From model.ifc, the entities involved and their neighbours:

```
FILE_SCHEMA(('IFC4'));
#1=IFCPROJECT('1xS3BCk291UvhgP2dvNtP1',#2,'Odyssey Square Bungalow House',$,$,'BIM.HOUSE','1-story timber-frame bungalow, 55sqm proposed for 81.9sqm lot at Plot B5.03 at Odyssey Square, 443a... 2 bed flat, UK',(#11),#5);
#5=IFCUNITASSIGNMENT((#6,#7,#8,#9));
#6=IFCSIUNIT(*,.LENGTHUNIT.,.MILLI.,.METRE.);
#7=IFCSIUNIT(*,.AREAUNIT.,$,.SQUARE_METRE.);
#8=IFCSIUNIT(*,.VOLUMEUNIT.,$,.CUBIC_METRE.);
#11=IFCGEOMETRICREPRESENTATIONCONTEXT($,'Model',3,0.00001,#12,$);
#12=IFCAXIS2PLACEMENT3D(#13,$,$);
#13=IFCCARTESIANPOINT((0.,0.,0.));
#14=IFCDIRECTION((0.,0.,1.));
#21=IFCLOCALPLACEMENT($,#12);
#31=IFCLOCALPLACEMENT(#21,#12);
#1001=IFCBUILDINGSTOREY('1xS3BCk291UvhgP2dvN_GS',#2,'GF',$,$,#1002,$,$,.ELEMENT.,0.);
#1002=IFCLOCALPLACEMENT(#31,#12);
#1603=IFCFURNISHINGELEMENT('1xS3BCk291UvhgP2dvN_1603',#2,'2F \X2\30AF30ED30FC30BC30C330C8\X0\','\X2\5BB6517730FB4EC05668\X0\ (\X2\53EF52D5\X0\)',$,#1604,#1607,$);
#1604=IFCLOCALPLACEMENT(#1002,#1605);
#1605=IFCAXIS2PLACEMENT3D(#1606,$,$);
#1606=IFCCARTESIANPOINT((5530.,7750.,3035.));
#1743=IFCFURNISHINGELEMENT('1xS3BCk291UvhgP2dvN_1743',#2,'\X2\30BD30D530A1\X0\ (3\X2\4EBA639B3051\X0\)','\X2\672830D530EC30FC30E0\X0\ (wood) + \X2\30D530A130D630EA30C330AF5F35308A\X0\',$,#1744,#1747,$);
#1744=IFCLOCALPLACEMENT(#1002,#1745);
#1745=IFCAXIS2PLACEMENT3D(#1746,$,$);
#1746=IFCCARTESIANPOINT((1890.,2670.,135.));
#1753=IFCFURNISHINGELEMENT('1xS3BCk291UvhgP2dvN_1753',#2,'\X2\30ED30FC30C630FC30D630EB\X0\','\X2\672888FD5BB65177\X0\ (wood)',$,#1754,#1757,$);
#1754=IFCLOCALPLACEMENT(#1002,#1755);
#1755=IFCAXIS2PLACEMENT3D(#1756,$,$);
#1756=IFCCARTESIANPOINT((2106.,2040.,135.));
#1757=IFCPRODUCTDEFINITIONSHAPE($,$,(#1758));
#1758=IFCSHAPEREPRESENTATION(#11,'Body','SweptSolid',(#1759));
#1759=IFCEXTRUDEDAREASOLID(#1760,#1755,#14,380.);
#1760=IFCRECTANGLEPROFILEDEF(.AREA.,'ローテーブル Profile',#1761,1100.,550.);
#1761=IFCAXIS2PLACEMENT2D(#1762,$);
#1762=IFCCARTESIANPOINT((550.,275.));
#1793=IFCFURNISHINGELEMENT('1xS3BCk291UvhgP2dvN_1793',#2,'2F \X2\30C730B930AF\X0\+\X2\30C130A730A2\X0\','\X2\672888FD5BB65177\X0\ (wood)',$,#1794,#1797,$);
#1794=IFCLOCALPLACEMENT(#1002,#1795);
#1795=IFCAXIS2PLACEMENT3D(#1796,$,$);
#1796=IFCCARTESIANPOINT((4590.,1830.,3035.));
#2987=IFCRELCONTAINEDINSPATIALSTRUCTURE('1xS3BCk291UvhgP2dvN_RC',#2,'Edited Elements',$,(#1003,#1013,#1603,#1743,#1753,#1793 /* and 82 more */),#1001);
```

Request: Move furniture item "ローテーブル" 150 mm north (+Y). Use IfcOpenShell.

```python
import ifcopenshell
import ifcopenshell.api.geometry
import ifcopenshell.util.placement

model = ifcopenshell.open("model.ifc")

item = model.by_guid("1xS3BCk291UvhgP2dvN_1753")
matrix = ifcopenshell.util.placement.get_local_placement(item.ObjectPlacement)
matrix[1, 3] += 150.0
ifcopenshell.api.geometry.edit_object_placement(model, product=item, matrix=matrix, is_si=False)

print(ifcopenshell.util.placement.get_local_placement(item.ObjectPlacement).round(3) + 0.0)

model.write("model_v2.ifc")
```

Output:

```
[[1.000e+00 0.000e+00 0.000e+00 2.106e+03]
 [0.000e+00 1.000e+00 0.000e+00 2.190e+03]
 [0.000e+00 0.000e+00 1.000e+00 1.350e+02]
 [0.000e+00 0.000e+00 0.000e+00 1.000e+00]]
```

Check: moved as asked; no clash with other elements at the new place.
